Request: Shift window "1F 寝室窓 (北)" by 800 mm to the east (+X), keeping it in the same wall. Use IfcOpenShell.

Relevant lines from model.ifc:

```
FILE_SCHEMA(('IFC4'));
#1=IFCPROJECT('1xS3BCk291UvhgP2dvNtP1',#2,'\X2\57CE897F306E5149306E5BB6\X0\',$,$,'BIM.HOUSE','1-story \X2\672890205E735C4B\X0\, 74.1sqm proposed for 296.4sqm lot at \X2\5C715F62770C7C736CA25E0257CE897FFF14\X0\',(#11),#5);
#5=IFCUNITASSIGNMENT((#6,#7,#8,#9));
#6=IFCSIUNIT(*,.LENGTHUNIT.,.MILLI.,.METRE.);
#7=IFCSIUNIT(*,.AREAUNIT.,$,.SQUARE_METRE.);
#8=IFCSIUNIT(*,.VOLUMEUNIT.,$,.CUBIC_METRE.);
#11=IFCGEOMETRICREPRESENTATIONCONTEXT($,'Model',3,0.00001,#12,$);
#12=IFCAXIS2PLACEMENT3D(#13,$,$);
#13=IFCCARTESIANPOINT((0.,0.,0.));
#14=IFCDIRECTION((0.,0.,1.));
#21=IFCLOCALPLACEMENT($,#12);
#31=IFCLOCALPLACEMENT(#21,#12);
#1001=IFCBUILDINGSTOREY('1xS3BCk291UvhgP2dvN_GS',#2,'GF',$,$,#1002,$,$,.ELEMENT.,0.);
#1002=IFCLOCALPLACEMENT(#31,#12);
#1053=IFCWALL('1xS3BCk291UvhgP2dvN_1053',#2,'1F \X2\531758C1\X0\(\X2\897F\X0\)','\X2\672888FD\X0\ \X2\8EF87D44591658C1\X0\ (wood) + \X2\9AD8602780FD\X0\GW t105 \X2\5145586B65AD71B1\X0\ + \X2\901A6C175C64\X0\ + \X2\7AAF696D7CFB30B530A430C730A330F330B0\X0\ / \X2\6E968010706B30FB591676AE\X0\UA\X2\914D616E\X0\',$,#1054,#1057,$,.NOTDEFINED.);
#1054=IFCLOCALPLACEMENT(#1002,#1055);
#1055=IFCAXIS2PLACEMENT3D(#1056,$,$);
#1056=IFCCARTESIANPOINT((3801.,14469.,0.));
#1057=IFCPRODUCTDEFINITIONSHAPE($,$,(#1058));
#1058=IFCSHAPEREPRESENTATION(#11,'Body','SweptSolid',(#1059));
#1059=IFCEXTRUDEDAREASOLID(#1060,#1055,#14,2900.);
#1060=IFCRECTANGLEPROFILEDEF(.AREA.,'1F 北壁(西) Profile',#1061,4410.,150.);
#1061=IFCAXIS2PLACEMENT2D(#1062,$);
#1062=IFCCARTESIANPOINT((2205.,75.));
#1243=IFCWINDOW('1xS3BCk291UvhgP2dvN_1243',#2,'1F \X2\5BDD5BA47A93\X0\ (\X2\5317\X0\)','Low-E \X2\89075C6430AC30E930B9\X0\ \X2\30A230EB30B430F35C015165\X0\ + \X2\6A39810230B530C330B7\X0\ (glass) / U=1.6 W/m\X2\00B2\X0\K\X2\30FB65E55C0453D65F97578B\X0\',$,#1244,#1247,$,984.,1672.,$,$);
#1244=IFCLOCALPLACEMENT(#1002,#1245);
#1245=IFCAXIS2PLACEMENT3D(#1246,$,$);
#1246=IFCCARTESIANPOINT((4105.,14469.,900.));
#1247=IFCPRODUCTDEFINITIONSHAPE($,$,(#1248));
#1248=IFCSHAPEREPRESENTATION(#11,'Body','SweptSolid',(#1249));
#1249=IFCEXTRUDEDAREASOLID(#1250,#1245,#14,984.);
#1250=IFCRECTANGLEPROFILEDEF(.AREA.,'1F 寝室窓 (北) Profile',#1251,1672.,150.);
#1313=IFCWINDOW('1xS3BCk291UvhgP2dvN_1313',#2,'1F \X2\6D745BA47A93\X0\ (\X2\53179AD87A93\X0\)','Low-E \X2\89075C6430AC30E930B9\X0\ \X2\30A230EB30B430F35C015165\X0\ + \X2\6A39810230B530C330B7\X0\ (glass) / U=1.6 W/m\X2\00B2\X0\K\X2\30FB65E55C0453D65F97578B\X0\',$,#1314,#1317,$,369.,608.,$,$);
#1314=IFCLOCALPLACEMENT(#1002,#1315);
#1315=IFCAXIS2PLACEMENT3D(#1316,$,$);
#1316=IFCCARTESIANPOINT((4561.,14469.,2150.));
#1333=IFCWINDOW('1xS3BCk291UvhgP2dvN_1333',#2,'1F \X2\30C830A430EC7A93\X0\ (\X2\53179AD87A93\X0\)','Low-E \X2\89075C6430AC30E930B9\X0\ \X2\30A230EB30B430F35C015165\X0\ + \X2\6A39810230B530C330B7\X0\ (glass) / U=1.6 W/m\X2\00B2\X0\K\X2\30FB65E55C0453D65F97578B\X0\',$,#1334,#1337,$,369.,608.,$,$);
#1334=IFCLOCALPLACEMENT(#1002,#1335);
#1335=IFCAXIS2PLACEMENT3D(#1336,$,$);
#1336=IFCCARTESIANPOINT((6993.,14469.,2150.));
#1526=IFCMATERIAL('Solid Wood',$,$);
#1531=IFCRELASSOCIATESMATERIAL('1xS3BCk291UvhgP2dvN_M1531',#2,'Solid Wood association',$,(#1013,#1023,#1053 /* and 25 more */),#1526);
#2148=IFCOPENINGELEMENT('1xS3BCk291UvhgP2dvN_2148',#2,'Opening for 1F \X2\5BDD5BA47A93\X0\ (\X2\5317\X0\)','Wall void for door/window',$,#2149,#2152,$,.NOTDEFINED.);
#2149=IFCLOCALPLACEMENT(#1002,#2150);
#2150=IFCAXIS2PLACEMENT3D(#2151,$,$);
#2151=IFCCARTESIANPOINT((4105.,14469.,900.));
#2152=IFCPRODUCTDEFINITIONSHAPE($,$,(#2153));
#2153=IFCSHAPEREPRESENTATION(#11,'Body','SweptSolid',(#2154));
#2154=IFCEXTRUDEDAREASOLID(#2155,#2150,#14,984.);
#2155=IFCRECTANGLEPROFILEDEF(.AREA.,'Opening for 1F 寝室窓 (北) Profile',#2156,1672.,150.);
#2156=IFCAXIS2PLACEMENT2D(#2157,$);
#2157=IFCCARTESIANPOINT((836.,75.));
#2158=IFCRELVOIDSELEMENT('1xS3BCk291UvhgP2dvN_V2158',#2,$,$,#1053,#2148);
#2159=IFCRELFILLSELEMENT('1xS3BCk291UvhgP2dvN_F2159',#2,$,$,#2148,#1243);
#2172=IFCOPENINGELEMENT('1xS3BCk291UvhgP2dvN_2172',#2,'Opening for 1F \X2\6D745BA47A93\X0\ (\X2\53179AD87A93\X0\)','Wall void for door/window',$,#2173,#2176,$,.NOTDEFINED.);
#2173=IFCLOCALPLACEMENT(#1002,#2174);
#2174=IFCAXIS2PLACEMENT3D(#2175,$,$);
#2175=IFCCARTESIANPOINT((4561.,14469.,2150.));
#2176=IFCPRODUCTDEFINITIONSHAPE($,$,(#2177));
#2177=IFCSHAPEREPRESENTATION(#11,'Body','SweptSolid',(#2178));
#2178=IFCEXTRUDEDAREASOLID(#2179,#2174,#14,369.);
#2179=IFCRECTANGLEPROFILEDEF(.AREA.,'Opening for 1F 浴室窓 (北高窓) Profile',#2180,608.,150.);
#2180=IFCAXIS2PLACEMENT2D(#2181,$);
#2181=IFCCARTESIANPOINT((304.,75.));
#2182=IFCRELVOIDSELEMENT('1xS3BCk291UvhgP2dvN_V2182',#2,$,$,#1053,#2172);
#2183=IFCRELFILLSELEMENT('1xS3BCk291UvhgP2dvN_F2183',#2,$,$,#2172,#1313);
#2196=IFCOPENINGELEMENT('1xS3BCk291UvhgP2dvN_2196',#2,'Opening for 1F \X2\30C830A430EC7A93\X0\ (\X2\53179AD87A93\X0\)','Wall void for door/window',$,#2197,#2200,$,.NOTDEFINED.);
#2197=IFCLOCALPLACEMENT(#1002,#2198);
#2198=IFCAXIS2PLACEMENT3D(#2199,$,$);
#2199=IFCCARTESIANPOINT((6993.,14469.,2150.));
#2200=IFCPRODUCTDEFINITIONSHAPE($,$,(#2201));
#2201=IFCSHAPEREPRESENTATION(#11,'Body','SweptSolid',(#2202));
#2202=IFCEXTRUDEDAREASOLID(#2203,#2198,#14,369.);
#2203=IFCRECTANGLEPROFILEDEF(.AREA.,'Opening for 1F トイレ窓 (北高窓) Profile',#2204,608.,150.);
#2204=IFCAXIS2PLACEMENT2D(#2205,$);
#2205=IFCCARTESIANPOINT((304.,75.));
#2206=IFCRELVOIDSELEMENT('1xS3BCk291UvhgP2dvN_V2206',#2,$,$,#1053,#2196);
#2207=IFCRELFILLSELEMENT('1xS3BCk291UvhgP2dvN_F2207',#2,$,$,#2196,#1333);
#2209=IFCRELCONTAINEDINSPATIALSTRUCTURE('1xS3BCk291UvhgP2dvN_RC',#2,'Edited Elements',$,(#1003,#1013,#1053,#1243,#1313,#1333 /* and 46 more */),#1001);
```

```python
import ifcopenshell
import ifcopenshell.api.geometry
import ifcopenshell.util.placement

model = ifcopenshell.open("model.ifc")

window = model.by_id(1243)
opening = window.FillsVoids[0].RelatingOpeningElement
wall = opening.VoidsElements[0].RelatingBuildingElement

wall_matrix = ifcopenshell.util.placement.get_local_placement(wall.ObjectPlacement)
shift = wall_matrix[:3, 0] * 800.0
before = ifcopenshell.util.placement.get_local_placement(window.ObjectPlacement)[:3, 3].copy()

# The window is not placed relative to its opening, so move both.
for product in (opening, window):
    matrix = ifcopenshell.util.placement.get_local_placement(product.ObjectPlacement)
    matrix[:3, 3] += shift
    ifcopenshell.api.geometry.edit_object_placement(model, product=product, matrix=matrix, is_si=False)

after = ifcopenshell.util.placement.get_local_placement(window.ObjectPlacement)[:3, 3]
print("window moved by", (after - before).round(3) + 0.0)

model.write("model-out.ifc")
```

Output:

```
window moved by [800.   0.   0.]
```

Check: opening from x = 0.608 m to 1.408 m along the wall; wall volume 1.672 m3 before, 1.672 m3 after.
